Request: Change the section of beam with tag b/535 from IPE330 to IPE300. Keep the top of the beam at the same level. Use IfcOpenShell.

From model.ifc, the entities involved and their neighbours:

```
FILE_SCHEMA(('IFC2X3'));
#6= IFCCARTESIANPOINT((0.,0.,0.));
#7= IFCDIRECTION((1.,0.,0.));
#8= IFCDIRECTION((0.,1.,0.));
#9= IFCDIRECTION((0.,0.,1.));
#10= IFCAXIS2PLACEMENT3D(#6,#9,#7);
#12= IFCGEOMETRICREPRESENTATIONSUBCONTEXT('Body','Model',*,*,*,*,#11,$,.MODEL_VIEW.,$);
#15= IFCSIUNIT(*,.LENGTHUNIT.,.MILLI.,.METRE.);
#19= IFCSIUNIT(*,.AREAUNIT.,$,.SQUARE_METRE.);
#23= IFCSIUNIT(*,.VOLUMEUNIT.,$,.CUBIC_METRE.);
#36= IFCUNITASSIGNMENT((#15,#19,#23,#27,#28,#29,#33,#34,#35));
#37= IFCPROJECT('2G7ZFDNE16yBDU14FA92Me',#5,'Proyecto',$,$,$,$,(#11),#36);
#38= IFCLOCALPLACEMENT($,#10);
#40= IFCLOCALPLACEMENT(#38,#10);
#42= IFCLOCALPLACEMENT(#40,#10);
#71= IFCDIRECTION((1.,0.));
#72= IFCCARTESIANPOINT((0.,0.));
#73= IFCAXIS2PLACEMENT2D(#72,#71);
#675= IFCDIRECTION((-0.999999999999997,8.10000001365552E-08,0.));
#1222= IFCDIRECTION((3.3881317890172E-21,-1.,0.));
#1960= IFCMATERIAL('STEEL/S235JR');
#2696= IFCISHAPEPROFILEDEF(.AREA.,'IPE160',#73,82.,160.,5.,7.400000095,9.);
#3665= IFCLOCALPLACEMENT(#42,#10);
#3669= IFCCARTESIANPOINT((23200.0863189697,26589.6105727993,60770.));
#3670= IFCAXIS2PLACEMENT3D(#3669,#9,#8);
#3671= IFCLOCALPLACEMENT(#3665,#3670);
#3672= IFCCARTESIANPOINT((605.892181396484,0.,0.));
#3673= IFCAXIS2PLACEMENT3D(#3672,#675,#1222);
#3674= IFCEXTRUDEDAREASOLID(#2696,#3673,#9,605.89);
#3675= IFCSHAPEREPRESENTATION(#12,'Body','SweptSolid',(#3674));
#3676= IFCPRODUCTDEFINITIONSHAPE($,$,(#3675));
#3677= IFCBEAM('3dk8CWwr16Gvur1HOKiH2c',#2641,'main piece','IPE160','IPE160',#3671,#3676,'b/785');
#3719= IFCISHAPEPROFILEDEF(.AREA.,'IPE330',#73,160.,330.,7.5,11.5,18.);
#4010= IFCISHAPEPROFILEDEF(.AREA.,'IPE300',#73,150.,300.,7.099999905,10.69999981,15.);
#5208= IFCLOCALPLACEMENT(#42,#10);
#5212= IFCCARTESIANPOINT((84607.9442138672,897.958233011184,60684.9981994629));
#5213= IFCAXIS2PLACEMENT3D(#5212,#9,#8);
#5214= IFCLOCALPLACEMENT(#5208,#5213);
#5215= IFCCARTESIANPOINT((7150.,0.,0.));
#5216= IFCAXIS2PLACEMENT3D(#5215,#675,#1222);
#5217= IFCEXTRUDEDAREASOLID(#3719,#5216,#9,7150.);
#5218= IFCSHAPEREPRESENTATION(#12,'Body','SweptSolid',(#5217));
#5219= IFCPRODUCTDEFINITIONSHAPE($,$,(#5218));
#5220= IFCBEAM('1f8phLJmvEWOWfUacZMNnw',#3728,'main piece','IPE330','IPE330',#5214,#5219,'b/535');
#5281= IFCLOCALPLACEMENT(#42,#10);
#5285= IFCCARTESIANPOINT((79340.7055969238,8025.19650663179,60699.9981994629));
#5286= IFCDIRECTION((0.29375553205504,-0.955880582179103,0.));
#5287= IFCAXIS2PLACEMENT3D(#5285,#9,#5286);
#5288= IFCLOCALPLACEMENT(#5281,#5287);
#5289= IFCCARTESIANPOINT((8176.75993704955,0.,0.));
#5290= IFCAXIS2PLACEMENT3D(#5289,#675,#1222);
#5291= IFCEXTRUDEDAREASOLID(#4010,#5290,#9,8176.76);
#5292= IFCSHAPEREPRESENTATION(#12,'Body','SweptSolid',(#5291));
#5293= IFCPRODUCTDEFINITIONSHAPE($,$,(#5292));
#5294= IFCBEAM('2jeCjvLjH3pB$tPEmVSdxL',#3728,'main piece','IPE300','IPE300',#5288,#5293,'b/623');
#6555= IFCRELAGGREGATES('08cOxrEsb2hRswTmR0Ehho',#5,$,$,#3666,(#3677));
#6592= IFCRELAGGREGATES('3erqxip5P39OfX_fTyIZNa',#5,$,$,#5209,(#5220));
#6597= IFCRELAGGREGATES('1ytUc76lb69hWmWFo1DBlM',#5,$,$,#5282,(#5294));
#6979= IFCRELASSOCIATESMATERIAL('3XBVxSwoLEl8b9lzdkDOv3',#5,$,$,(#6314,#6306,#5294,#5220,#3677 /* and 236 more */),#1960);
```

```python
import ifcopenshell
import ifcopenshell.util.element
import ifcopenshell.util.representation

model = ifcopenshell.open("model.ifc")

member = model.by_guid("1f8phLJmvEWOWfUacZMNnw")
source = next(p for p in model.by_type("IfcIShapeProfileDef") if p.ProfileName == "IPE300")

body = ifcopenshell.util.representation.get_representation(member, "Model", "Body")
solid = body.Items[0]
old_profile = solid.SweptArea

# Copy the section's sizes but keep this member's own profile position.
profile = ifcopenshell.util.element.copy(model, source)
# Profiles are centred, so shift by half the change in depth to hold the top.
shift = (old_profile.OverallDepth - profile.OverallDepth) / 2
x, y = old_profile.Position.Location.Coordinates
up = (0.0, 1.0)  # upwards, in the solid's own plane
location = model.createIfcCartesianPoint((x + up[0] * shift, y + up[1] * shift))
profile.Position = model.createIfcAxis2Placement2D(location, old_profile.Position.RefDirection)
solid.SweptArea = profile
if not model.get_total_inverses(old_profile):
    ifcopenshell.util.element.remove_deep2(model, old_profile)
member.Description = member.Description.replace("IPE330", "IPE300")
member.ObjectType = member.ObjectType.replace("IPE330", "IPE300")

print(solid.SweptArea)

model.write("model_rev.ifc")
```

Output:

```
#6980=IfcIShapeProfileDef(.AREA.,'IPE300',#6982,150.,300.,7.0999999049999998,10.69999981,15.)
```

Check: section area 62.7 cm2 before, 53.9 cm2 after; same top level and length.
